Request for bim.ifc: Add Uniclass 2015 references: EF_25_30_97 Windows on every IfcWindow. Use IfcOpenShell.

First a look at what the model holds.

```python
import ifcopenshell

model = ifcopenshell.open("bim.ifc")
print(model.schema)
print("classifications:", [c.Name for c in model.by_type("IfcClassification")])
for ifc_class in ("IfcDoor", "IfcRoof", "IfcStair", "IfcWall", "IfcWindow"):
    print(ifc_class, len(model.by_type(ifc_class)))
```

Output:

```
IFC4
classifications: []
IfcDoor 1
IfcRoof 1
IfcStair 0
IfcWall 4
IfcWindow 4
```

```python
import ifcopenshell
import ifcopenshell.api.classification

model = ifcopenshell.open("bim.ifc")

system = ifcopenshell.api.classification.add_classification(model, classification="Uniclass 2015")

codes = {
    "IfcWindow": ("EF_25_30_97", "Windows"),
}
for ifc_class, (code, name) in codes.items():
    products = model.by_type(ifc_class)
    ifcopenshell.api.classification.add_reference(
        model, products=products, classification=system, identification=code, name=name
    )
    print(code, len(products))

model.write("bim-out.ifc")
```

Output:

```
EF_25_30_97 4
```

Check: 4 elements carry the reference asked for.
